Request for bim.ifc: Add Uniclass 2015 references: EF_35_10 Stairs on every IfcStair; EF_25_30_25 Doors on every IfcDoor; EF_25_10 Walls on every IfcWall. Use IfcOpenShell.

First a look at what the model holds.

```python
import ifcopenshell

model = ifcopenshell.open("bim.ifc")
print(model.schema)
print("classifications:", [c.Name for c in model.by_type("IfcClassification")])
for ifc_class in ("IfcDoor", "IfcRoof", "IfcStair", "IfcWall", "IfcWindow"):
    print(ifc_class, len(model.by_type(ifc_class)))
```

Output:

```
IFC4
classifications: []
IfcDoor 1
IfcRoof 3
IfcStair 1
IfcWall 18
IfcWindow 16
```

```python
import ifcopenshell
import ifcopenshell.api.classification

model = ifcopenshell.open("bim.ifc")

system = ifcopenshell.api.classification.add_classification(model, classification="Uniclass 2015")

codes = {
    "IfcStair": ("EF_35_10", "Stairs"),
    "IfcDoor": ("EF_25_30_25", "Doors"),
    "IfcWall": ("EF_25_10", "Walls"),
}
for ifc_class, (code, name) in codes.items():
    products = model.by_type(ifc_class)
    ifcopenshell.api.classification.add_reference(
        model, products=products, classification=system, identification=code, name=name
    )
    print(code, len(products))

model.write("bim-out.ifc")
```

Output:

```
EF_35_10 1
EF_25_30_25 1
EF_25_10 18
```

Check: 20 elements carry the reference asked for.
